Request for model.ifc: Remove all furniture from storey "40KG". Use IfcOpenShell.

First a look at what the model holds.

```python
import ifcopenshell
import ifcopenshell.util.element

model = ifcopenshell.open("model.ifc")
print(model.schema)
storey = next(s for s in model.by_type("IfcBuildingStorey") if s.Name == "40KG")
furniture = [e for e in ifcopenshell.util.element.get_decomposition(storey) if e.is_a("IfcFurnishingElement")]
seen = {}
for e in furniture:
    element_type = ifcopenshell.util.element.get_type(e)
    name = element_type.Name if element_type not in (None, e) else None
    seen[name] = seen.get(name, 0) + 1
for name, count in sorted(seen.items(), key=str):
    print(count, "x", name)
```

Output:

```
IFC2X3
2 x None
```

```python
import ifcopenshell
import ifcopenshell.api.root
import ifcopenshell.util.element

model = ifcopenshell.open("model.ifc")

storey = next(s for s in model.by_type("IfcBuildingStorey") if s.Name == "40KG")
furniture = [e for e in ifcopenshell.util.element.get_decomposition(storey) if e.is_a("IfcFurnishingElement")]

for e in furniture:
    ifcopenshell.api.root.remove_product(model, product=e)
print(len(furniture), "removed")

model.write("model-out.ifc")
```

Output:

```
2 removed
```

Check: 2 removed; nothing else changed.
